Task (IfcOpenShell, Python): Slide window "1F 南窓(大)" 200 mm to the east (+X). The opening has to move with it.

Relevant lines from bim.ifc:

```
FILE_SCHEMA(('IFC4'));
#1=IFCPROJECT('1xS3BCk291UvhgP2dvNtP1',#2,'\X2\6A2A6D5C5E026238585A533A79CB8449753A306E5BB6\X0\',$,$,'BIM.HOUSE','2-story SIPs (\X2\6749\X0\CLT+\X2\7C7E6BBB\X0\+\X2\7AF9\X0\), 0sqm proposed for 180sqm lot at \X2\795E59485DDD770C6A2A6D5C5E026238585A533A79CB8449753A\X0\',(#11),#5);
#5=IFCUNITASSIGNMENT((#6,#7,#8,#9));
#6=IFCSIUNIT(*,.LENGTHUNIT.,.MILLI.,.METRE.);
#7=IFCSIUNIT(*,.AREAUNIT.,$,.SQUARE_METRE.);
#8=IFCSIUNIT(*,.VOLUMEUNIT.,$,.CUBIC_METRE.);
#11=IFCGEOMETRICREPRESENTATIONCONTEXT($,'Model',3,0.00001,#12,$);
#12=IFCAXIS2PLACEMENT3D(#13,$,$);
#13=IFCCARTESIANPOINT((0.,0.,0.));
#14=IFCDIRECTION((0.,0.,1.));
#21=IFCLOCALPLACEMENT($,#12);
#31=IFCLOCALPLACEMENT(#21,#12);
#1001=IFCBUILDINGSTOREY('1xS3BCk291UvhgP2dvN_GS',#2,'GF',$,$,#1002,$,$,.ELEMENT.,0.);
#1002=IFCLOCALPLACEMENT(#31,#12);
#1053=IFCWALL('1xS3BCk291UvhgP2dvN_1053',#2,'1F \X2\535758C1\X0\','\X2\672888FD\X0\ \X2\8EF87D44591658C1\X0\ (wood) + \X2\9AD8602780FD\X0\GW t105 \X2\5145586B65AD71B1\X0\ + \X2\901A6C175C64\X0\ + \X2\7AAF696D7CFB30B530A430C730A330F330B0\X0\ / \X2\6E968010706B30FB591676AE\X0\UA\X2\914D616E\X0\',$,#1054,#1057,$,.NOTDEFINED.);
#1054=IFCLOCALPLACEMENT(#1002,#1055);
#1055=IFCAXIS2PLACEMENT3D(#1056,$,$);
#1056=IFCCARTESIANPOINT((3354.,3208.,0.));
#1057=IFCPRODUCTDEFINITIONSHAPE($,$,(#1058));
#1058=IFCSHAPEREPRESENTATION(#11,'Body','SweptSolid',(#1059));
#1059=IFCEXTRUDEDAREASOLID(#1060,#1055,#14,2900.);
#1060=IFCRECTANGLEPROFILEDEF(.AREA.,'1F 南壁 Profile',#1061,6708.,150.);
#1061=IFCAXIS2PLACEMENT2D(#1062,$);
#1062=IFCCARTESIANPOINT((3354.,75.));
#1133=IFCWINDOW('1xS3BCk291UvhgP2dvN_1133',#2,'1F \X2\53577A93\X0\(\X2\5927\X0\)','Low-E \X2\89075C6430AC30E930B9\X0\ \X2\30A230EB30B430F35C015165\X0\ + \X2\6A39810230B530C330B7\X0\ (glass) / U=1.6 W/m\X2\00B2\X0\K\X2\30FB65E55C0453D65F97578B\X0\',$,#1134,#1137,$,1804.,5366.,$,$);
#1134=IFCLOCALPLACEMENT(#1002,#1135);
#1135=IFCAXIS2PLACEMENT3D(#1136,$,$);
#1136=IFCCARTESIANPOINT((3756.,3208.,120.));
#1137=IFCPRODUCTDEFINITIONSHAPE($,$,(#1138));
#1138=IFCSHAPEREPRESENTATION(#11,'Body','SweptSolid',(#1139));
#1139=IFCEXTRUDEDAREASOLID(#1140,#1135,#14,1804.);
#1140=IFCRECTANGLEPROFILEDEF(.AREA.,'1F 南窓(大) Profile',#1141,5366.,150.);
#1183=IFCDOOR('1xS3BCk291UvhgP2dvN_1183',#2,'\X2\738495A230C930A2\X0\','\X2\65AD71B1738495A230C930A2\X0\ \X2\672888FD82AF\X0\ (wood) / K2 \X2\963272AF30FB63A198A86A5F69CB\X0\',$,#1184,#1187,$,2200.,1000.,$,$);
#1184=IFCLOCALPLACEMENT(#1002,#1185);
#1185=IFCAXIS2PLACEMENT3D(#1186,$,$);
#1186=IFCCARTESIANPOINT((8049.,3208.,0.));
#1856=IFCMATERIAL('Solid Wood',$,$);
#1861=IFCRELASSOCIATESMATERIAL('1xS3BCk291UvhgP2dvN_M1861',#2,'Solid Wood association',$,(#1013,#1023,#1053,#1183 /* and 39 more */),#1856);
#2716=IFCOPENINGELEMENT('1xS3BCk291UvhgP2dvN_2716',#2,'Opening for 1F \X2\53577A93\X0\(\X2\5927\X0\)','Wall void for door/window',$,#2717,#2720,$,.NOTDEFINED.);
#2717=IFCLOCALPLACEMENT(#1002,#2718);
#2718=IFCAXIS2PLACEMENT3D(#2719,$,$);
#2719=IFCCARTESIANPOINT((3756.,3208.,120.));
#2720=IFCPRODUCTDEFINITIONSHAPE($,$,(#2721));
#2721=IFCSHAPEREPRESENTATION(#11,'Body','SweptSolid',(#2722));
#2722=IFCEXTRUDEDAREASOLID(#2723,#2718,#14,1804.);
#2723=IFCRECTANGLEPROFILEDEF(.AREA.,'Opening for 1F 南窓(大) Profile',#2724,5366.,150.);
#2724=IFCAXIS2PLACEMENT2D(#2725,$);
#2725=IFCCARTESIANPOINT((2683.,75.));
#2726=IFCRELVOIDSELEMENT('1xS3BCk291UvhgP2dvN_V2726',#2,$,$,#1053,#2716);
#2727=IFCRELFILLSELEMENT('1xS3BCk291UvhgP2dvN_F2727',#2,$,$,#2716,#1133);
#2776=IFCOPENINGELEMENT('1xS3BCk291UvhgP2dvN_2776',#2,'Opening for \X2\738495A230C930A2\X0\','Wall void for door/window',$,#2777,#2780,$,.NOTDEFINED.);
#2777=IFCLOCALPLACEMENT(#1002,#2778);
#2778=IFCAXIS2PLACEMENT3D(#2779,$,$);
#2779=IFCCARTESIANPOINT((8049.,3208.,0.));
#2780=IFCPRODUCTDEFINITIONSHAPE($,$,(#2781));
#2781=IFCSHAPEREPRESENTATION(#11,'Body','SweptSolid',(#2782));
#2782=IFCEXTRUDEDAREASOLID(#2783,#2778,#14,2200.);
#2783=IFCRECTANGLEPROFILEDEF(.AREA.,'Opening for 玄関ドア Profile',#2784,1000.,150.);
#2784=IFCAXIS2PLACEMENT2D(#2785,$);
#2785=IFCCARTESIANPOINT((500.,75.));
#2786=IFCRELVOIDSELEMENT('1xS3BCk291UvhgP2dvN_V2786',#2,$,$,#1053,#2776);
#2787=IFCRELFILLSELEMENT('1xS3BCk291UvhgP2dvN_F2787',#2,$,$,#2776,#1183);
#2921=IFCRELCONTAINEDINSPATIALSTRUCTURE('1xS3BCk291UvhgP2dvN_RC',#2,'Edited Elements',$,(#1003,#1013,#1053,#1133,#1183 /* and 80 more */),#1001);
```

```python
import ifcopenshell
import ifcopenshell.api.geometry
import ifcopenshell.util.placement

model = ifcopenshell.open("bim.ifc")

window = model.by_guid("1xS3BCk291UvhgP2dvN_1133")
opening = window.FillsVoids[0].RelatingOpeningElement
wall = opening.VoidsElements[0].RelatingBuildingElement

wall_matrix = ifcopenshell.util.placement.get_local_placement(wall.ObjectPlacement)
shift = wall_matrix[:3, 0] * 200.0
before = ifcopenshell.util.placement.get_local_placement(window.ObjectPlacement)[:3, 3].copy()

# The window is not placed relative to its opening, so move both.
for product in (opening, window):
    matrix = ifcopenshell.util.placement.get_local_placement(product.ObjectPlacement)
    matrix[:3, 3] += shift
    ifcopenshell.api.geometry.edit_object_placement(model, product=product, matrix=matrix, is_si=False)

after = ifcopenshell.util.placement.get_local_placement(window.ObjectPlacement)[:3, 3]
print("window moved by", (after - before).round(3) + 0.0)

model.write("bim_v2.ifc")
```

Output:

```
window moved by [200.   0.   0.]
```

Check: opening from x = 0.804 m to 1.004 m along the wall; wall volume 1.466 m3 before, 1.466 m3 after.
